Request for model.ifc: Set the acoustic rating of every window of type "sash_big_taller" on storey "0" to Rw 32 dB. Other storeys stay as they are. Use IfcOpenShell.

First a look at what the model holds.

```python
import ifcopenshell
import ifcopenshell.util.element

model = ifcopenshell.open("model.ifc")
print(model.schema)
storey = next(s for s in model.by_type("IfcBuildingStorey") if s.Name == "0")
windows = [e for e in ifcopenshell.util.element.get_decomposition(storey) if e.is_a("IfcWindow")]
seen = {}
for e in windows:
    element_type = ifcopenshell.util.element.get_type(e)
    key = (element_type.Name if element_type != e and element_type else None, ifcopenshell.util.element.get_pset(e, "Pset_WindowCommon", "AcousticRating"))
    seen[key] = seen.get(key, 0) + 1
for (name, value), count in sorted(seen.items(), key=str):
    print(count, "x", name, "|", value)
```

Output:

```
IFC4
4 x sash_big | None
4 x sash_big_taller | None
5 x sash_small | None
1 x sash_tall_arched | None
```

```python
import ifcopenshell
import ifcopenshell.api.pset
import ifcopenshell.util.element

model = ifcopenshell.open("model.ifc")

storey = next(s for s in model.by_type("IfcBuildingStorey") if s.Name == "0")
windows = [e for e in ifcopenshell.util.element.get_decomposition(storey) if e.is_a("IfcWindow")]

count = 0
for e in windows:
    element_type = ifcopenshell.util.element.get_type(e)
    if element_type in (None, e) or element_type.Name != "sash_big_taller":
        continue
    # add_pset returns the element's existing set when there is one.
    pset = ifcopenshell.api.pset.add_pset(model, product=e, name="Pset_WindowCommon")
    ifcopenshell.api.pset.edit_pset(model, pset=pset, properties={"AcousticRating": "Rw 32 dB"})
    count += 1

print(count, "windows updated")

model.write("model_v2.ifc")
```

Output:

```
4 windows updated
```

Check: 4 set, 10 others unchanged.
